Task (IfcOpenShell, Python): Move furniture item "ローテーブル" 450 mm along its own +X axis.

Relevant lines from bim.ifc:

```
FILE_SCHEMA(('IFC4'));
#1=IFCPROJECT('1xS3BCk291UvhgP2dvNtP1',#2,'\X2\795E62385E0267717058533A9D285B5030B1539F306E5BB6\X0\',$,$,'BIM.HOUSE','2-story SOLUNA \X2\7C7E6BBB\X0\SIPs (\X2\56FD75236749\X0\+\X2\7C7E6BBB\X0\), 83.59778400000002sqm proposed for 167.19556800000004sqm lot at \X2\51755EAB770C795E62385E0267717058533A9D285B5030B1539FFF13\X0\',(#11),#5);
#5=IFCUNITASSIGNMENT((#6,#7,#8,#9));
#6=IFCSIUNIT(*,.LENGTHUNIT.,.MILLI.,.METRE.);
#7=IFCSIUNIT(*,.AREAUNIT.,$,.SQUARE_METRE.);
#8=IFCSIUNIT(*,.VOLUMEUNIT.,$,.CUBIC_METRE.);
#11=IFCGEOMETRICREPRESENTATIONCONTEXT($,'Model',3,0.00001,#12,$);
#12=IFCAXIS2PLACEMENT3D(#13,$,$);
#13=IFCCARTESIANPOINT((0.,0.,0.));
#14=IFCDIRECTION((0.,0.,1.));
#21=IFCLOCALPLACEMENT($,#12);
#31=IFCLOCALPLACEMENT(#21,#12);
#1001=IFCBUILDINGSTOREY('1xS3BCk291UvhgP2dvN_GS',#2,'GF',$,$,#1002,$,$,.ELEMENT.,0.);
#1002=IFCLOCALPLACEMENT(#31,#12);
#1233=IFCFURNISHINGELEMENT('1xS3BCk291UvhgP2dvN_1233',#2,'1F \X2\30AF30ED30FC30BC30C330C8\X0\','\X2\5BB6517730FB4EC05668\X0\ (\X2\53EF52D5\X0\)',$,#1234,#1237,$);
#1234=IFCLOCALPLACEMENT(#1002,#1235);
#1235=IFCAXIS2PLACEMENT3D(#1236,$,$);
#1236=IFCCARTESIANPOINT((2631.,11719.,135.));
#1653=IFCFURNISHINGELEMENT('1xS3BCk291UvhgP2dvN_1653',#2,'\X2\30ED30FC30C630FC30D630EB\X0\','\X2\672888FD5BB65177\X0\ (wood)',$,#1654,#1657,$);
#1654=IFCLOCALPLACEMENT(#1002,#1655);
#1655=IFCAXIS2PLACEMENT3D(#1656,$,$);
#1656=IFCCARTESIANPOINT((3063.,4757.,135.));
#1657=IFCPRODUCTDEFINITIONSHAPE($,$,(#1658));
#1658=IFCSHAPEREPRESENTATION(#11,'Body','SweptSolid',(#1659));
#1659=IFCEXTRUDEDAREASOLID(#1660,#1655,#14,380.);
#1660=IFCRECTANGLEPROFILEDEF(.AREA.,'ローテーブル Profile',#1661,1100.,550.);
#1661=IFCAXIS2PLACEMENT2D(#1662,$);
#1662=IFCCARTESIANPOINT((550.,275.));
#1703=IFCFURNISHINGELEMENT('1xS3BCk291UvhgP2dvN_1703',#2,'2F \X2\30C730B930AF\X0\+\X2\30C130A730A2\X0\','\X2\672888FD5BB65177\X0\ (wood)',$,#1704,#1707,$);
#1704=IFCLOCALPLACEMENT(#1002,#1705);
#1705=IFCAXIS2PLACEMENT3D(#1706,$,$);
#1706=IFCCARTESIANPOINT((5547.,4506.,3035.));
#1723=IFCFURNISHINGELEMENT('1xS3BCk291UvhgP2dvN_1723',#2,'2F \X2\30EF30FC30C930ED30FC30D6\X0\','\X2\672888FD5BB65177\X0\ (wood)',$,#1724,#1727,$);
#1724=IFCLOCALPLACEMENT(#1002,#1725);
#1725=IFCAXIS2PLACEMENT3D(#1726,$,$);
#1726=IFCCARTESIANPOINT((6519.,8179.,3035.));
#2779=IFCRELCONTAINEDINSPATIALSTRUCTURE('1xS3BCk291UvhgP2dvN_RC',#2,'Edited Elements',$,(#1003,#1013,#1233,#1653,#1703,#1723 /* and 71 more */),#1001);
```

```python
import ifcopenshell
import ifcopenshell.api.geometry
import ifcopenshell.util.placement
import ifcopenshell.util.unit

model = ifcopenshell.open("bim.ifc")
unit_scale = ifcopenshell.util.unit.calculate_unit_scale(model)

item = model.by_guid("1xS3BCk291UvhgP2dvN_1653")
matrix = ifcopenshell.util.placement.get_local_placement(item.ObjectPlacement)
matrix[:3, 3] += matrix[:3, 0] * 0.45 / unit_scale
ifcopenshell.api.geometry.edit_object_placement(model, product=item, matrix=matrix, is_si=False)

print(ifcopenshell.util.placement.get_local_placement(item.ObjectPlacement).round(3) + 0.0)

model.write("bim-out.ifc")
```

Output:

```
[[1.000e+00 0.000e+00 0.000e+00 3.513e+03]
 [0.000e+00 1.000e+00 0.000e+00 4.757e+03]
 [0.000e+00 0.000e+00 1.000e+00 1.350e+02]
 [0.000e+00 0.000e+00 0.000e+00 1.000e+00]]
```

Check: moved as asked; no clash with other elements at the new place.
